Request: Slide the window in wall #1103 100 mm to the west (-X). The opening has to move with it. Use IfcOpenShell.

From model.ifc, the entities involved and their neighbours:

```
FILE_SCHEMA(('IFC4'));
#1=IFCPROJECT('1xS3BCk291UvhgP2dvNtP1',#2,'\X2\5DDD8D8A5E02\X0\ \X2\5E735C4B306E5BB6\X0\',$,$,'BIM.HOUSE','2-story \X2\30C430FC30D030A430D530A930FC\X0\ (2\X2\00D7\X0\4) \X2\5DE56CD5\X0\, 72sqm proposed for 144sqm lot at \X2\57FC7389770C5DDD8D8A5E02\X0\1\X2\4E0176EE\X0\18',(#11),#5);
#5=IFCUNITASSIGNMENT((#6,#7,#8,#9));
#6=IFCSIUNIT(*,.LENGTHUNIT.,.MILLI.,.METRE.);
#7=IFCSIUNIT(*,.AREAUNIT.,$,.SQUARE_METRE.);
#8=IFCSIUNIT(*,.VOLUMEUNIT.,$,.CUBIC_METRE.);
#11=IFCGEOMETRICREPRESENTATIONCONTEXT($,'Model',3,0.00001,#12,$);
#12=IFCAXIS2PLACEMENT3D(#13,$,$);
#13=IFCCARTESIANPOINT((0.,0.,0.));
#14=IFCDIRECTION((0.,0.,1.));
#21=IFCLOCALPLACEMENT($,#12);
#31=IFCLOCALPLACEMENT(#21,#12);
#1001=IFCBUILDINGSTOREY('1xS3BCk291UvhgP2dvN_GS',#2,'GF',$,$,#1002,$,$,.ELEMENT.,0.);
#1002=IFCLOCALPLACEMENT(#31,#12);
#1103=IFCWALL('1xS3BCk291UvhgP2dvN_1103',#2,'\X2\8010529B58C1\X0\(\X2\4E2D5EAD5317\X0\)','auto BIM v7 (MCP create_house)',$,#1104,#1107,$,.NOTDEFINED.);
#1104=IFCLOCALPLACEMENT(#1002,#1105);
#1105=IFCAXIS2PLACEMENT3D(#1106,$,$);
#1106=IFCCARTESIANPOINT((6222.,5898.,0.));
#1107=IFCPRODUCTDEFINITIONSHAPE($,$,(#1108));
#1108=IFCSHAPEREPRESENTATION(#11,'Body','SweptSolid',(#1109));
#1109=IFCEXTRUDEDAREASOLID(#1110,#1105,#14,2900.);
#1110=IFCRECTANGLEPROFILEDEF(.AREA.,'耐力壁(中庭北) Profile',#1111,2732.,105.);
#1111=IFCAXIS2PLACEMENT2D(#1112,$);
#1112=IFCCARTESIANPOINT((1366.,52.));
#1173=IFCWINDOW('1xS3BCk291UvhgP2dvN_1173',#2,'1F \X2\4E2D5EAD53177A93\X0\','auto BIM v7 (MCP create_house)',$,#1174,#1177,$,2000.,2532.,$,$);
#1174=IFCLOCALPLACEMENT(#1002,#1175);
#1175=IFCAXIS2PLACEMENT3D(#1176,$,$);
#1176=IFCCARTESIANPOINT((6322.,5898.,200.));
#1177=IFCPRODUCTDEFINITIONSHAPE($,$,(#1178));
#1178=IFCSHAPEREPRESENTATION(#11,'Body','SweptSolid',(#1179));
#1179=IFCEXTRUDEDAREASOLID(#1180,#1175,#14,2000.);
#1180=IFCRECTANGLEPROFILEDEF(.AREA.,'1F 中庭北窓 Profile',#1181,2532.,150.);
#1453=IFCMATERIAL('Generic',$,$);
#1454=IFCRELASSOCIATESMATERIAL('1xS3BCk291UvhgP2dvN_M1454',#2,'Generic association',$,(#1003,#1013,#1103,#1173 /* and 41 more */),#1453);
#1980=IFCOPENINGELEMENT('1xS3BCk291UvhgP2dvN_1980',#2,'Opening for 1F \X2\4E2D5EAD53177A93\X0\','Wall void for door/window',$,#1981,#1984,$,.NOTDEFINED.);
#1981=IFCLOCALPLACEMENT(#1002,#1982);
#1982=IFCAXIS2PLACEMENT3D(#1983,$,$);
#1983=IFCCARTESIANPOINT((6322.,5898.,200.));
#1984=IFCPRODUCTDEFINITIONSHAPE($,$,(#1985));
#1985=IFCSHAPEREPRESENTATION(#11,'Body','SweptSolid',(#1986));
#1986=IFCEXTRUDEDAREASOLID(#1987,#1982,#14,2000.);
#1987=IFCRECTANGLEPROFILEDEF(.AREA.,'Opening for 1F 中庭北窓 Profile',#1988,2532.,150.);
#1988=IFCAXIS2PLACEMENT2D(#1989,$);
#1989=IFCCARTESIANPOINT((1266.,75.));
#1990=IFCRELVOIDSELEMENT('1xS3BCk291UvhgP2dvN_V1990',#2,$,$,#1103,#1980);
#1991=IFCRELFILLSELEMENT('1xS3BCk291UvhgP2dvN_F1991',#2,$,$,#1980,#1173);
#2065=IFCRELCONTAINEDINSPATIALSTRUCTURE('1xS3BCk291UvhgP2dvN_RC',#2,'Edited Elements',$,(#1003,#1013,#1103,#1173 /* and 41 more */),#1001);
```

```python
import ifcopenshell
import ifcopenshell.api.geometry
import ifcopenshell.util.placement
import ifcopenshell.util.unit

model = ifcopenshell.open("model.ifc")
unit_scale = ifcopenshell.util.unit.calculate_unit_scale(model)

window = model.by_id(1173)
opening = window.FillsVoids[0].RelatingOpeningElement
wall = opening.VoidsElements[0].RelatingBuildingElement

wall_matrix = ifcopenshell.util.placement.get_local_placement(wall.ObjectPlacement)
shift = wall_matrix[:3, 0] * -0.1 / unit_scale
before = ifcopenshell.util.placement.get_local_placement(window.ObjectPlacement)[:3, 3].copy()

# The window is not placed relative to its opening, so move both.
for product in (opening, window):
    matrix = ifcopenshell.util.placement.get_local_placement(product.ObjectPlacement)
    matrix[:3, 3] += shift
    ifcopenshell.api.geometry.edit_object_placement(model, product=product, matrix=matrix, is_si=False)

after = ifcopenshell.util.placement.get_local_placement(window.ObjectPlacement)[:3, 3]
print("window moved by", (after - before).round(3) + 0.0)

model.write("model_edited.ifc")
```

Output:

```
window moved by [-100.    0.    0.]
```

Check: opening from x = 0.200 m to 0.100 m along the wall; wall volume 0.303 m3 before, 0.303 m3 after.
